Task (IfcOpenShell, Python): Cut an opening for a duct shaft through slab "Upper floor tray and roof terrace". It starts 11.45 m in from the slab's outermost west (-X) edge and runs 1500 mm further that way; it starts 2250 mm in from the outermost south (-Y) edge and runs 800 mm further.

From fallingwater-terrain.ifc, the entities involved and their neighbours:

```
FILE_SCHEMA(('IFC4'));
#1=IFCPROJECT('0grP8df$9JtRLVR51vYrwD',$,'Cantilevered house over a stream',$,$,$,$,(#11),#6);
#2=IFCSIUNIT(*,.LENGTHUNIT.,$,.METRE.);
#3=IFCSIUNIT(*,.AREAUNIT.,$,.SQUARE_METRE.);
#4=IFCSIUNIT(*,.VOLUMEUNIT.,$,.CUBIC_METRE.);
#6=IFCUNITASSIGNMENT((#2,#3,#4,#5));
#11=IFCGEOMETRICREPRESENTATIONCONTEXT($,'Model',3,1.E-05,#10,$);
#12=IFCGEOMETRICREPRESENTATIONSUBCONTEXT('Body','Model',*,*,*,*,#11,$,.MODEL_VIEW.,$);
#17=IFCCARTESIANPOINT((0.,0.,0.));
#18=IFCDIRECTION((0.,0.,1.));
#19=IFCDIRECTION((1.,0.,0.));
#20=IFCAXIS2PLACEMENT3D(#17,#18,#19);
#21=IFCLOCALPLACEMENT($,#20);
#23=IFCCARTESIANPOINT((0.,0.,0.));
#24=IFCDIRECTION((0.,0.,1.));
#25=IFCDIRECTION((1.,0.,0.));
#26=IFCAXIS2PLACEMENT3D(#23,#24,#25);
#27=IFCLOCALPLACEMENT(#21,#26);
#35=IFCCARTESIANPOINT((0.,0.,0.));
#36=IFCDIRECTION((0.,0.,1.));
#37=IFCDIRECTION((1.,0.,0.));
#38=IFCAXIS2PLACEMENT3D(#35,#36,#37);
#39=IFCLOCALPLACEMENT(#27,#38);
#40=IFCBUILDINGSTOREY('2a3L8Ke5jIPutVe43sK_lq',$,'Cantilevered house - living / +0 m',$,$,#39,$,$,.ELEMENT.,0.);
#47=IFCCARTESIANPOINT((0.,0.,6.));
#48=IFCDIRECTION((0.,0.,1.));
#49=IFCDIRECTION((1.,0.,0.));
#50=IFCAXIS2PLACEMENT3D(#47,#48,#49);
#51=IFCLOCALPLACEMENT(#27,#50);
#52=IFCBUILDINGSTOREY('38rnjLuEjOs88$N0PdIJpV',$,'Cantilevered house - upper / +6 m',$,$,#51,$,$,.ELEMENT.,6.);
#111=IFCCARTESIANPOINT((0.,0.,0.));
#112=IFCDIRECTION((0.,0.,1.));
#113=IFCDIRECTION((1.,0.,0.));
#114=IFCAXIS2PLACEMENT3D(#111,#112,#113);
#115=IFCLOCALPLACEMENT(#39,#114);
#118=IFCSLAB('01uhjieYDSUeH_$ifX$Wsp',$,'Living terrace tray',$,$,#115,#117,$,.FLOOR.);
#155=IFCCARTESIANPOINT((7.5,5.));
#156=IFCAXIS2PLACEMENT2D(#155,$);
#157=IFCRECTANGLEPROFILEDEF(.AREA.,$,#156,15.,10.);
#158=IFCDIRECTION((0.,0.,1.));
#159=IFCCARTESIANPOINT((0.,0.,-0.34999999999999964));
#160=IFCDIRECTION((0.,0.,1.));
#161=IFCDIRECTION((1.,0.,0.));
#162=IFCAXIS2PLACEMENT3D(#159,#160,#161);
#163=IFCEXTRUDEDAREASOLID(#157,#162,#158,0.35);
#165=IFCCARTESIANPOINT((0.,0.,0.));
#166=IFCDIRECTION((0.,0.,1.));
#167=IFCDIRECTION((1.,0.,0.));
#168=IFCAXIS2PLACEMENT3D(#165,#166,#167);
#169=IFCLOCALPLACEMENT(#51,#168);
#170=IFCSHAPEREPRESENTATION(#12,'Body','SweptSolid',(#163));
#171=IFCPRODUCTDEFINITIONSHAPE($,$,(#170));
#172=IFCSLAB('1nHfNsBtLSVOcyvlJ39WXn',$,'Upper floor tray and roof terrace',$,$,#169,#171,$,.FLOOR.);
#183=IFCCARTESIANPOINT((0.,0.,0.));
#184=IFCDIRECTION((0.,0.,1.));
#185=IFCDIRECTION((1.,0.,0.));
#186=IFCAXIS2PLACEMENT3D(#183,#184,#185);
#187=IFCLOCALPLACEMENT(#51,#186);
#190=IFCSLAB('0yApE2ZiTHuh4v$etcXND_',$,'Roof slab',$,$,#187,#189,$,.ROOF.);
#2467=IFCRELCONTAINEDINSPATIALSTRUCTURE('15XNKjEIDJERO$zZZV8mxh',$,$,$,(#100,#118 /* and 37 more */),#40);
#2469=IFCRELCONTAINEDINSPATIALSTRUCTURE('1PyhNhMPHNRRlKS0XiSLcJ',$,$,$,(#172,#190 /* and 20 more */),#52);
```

```python
import numpy as np
import ifcopenshell
import ifcopenshell.api.feature
import ifcopenshell.api.geometry
import ifcopenshell.api.root
import ifcopenshell.geom
import ifcopenshell.util.placement
import ifcopenshell.util.representation
import ifcopenshell.util.shape
import ifcopenshell.util.unit

model = ifcopenshell.open("fallingwater-terrain.ifc")
unit_scale = ifcopenshell.util.unit.calculate_unit_scale(model)
settings = ifcopenshell.geom.settings()


def volume(element):
    """Net volume in cubic metres, openings subtracted."""
    shape = ifcopenshell.geom.create_shape(settings, element)
    return ifcopenshell.util.shape.get_volume(shape.geometry)


slab = model.by_id(172)
before = volume(slab)

# Extent in the slab's own axes, in metres. The edges named are its -X and -Y sides.
slab_shape = ifcopenshell.geom.create_shape(settings, slab)
vertices = ifcopenshell.util.shape.get_vertices(slab_shape.geometry)
x_min, y_min, bottom = vertices.min(axis=0)
top = vertices[:, 2].max()

opening = ifcopenshell.api.root.create_entity(model, ifc_class="IfcOpeningElement", name="Duct shaft opening", predefined_type="OPENING")
context = ifcopenshell.util.representation.get_context(model, "Model", "Body", "MODEL_VIEW")
width, depth = 1.5, 0.8
outline = [(0.0, 0.0), (width, 0.0), (width, depth), (0.0, depth), (0.0, 0.0)]
# Overshoot both faces by 50 mm so the cut is clean.
shape = ifcopenshell.api.geometry.add_slab_representation(
    model, context=context, depth=top - bottom + 0.1, polyline=outline
)
ifcopenshell.api.geometry.assign_representation(model, product=opening, representation=shape)

matrix = ifcopenshell.util.placement.get_local_placement(slab.ObjectPlacement)
matrix[:, 3] = matrix @ np.append(np.array([x_min + 11.45, y_min + 2.25, bottom - 0.05]) / unit_scale, 1.0)
ifcopenshell.api.geometry.edit_object_placement(model, product=opening, matrix=matrix, is_si=False)
ifcopenshell.api.feature.add_feature(model, feature=opening, element=slab)

after = volume(slab)

print(f"slab volume {before:.3f} -> {after:.3f} m3")

model.write("fallingwater-terrain_updated.ifc")
```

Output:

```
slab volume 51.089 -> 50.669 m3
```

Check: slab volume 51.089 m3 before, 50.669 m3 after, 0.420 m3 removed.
